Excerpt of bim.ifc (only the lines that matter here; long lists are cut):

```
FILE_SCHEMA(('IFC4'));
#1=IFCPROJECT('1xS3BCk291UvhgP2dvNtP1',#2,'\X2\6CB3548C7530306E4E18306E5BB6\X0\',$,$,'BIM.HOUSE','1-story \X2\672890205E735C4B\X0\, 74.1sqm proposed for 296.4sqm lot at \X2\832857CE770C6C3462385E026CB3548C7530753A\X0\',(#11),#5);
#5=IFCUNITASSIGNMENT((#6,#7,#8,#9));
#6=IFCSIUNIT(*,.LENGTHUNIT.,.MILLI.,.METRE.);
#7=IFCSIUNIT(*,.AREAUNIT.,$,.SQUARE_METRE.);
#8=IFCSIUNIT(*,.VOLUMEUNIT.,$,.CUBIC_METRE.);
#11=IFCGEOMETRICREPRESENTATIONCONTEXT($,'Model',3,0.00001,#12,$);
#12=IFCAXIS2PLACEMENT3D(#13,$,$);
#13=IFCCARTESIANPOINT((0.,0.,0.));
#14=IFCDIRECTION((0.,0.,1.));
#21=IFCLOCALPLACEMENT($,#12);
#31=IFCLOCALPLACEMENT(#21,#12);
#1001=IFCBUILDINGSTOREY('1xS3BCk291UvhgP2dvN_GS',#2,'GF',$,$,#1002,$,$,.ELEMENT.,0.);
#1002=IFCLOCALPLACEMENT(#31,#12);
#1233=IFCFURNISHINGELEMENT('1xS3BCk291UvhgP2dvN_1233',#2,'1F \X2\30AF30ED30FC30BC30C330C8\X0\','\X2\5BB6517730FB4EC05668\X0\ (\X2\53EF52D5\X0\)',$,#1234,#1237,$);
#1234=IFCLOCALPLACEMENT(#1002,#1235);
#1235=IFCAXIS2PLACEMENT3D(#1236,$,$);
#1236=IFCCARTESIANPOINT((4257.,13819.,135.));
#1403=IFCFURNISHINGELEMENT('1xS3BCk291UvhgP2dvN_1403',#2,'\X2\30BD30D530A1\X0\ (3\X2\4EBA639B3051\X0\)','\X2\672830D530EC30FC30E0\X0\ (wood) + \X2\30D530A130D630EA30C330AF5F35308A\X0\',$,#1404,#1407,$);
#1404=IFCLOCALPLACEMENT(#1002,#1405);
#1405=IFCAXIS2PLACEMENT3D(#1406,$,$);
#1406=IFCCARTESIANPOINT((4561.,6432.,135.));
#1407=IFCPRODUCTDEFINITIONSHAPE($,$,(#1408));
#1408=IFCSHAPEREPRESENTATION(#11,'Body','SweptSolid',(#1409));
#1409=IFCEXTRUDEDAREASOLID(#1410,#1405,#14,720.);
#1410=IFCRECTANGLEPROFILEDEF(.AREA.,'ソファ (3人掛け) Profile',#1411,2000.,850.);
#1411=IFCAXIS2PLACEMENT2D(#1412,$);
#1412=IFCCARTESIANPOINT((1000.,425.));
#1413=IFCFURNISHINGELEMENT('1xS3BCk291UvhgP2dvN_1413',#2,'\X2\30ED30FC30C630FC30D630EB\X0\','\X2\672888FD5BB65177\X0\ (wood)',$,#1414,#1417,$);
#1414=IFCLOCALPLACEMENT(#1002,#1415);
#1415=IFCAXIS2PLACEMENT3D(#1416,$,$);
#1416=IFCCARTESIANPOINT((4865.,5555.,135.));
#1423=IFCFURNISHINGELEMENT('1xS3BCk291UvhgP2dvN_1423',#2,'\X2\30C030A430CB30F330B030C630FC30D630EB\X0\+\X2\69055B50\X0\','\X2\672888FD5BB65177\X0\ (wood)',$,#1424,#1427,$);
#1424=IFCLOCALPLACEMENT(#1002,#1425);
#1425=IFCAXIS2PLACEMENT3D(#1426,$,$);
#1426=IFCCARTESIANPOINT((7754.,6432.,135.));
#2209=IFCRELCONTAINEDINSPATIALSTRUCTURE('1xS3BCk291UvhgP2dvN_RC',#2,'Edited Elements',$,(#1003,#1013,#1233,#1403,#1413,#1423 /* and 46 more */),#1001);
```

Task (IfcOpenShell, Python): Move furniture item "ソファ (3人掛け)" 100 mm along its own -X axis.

```python
import ifcopenshell
import ifcopenshell.api.geometry
import ifcopenshell.util.placement
import ifcopenshell.util.unit

model = ifcopenshell.open("bim.ifc")
unit_scale = ifcopenshell.util.unit.calculate_unit_scale(model)

item = model.by_guid("1xS3BCk291UvhgP2dvN_1403")
matrix = ifcopenshell.util.placement.get_local_placement(item.ObjectPlacement)
matrix[:3, 3] -= matrix[:3, 0] * 0.1 / unit_scale
ifcopenshell.api.geometry.edit_object_placement(model, product=item, matrix=matrix, is_si=False)

print(ifcopenshell.util.placement.get_local_placement(item.ObjectPlacement).round(3) + 0.0)

model.write("bim_edited.ifc")
```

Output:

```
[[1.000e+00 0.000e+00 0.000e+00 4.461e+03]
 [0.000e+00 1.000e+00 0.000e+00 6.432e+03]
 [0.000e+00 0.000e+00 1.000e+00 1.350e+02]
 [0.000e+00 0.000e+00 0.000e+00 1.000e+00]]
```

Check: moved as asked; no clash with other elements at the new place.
